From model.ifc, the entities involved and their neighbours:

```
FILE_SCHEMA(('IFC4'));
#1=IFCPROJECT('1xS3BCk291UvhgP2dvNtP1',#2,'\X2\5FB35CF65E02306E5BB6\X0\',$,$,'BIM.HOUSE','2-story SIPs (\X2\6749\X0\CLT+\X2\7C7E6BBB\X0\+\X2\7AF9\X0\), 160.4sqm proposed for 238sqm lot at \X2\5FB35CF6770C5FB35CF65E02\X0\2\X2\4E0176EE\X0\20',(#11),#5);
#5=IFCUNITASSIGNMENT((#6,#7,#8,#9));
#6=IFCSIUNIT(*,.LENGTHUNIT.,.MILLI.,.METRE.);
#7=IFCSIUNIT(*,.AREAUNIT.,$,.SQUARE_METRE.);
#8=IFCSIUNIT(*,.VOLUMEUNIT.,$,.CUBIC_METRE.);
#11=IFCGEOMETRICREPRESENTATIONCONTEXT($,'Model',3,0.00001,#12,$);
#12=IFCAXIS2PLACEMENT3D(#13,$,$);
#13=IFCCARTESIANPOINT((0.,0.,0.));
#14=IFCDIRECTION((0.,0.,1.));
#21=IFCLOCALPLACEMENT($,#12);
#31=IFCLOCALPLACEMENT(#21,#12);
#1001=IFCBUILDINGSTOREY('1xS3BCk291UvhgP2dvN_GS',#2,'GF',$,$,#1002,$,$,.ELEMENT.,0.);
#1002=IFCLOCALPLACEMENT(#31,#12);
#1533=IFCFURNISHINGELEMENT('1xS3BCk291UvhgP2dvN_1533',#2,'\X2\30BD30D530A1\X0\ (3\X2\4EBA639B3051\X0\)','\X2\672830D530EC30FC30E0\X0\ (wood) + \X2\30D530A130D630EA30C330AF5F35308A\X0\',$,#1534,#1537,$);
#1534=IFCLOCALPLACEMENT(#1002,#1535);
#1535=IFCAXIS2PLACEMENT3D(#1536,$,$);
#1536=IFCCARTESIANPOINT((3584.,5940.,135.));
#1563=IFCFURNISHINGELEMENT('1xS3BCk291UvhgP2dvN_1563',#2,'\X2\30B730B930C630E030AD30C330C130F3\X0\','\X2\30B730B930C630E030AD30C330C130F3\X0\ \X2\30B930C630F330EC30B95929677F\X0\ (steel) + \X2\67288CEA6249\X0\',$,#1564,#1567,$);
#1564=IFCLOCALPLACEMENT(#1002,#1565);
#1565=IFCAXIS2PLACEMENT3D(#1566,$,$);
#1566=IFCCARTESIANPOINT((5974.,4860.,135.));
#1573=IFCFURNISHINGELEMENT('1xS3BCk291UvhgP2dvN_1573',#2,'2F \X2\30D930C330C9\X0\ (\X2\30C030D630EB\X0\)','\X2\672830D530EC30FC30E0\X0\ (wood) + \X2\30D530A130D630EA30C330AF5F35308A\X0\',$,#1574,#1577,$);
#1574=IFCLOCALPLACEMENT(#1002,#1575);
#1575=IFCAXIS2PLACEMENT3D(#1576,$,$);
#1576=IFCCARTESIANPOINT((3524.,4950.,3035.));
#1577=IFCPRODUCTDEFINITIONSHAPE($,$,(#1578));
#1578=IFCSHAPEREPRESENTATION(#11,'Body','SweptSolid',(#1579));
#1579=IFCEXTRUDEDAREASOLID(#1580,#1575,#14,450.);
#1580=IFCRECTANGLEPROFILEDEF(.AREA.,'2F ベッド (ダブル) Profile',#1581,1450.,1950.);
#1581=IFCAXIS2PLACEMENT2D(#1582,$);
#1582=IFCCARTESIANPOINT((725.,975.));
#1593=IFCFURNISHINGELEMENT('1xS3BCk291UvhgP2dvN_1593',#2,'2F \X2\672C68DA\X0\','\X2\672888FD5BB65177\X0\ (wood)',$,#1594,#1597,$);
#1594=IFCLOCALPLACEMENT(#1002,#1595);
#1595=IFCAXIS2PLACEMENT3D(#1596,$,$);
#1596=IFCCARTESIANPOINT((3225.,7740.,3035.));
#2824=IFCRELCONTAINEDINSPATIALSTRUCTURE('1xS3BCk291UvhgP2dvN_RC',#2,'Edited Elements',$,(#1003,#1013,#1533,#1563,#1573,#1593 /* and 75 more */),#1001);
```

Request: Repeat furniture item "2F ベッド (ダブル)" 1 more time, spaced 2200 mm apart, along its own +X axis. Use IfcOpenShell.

```python
import ifcopenshell
import ifcopenshell.api.geometry
import ifcopenshell.api.root
import ifcopenshell.util.element
import ifcopenshell.util.placement

model = ifcopenshell.open("model.ifc")


def reuse_history(source, copy):
    """copy_class also copies each property set's owner history, people and application; keep the originals."""
    for rel in copy.IsDefinedBy:
        if rel.is_a("IfcRelDefinesByProperties") and (history := rel.RelatingPropertyDefinition.OwnerHistory):
            rel.RelatingPropertyDefinition.OwnerHistory = source.OwnerHistory
            ifcopenshell.util.element.remove_deep2(model, history)


source = model.by_guid("1xS3BCk291UvhgP2dvN_1573")
base = ifcopenshell.util.placement.get_local_placement(source.ObjectPlacement)
step = base[:3, 0] * 2200.0

for i in range(1, 2):
    copy = ifcopenshell.api.root.copy_class(model, product=source)
    copy.Representation = ifcopenshell.util.element.copy_deep(
        model, source.Representation, exclude=["IfcGeometricRepresentationContext", "IfcRepresentationMap"]
    )
    reuse_history(source, copy)
    matrix = base.copy()
    matrix[:3, 3] += i * step
    print("added at", matrix[:3, 3].round(3) + 0.0)
    ifcopenshell.api.geometry.edit_object_placement(model, product=copy, matrix=matrix, is_si=False)

model.write("model-out.ifc")
```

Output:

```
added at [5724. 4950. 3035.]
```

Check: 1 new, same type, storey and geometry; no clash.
